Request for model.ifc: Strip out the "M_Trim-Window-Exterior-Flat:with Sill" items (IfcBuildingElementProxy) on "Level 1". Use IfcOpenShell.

First a look at what the model holds.

```python
import ifcopenshell
import ifcopenshell.util.element

model = ifcopenshell.open("model.ifc")
print(model.schema)
storey = next(s for s in model.by_type("IfcBuildingStorey") if s.Name == "Level 1")
proxies = [e for e in ifcopenshell.util.element.get_decomposition(storey) if e.is_a("IfcBuildingElementProxy")]
seen = {}
for e in proxies:
    element_type = ifcopenshell.util.element.get_type(e)
    name = element_type.Name if element_type not in (None, e) else None
    seen[name] = seen.get(name, 0) + 1
for name, count in sorted(seen.items(), key=str):
    print(count, "x", name)
```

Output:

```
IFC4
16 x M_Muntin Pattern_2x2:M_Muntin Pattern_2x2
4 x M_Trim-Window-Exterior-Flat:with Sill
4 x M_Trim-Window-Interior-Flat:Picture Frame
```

```python
import ifcopenshell
import ifcopenshell.api.root
import ifcopenshell.util.element

model = ifcopenshell.open("model.ifc")

storey = next(s for s in model.by_type("IfcBuildingStorey") if s.Name == "Level 1")
proxies = [e for e in ifcopenshell.util.element.get_decomposition(storey) if e.is_a("IfcBuildingElementProxy")]
targets = [e for e in proxies if (t := ifcopenshell.util.element.get_type(e)) not in (None, e) and t.Name == "M_Trim-Window-Exterior-Flat:with Sill"]

for e in targets:
    ifcopenshell.api.root.remove_product(model, product=e)
print(len(targets), "removed")

model.write("model_v2.ifc")
```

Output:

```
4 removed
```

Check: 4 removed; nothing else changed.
